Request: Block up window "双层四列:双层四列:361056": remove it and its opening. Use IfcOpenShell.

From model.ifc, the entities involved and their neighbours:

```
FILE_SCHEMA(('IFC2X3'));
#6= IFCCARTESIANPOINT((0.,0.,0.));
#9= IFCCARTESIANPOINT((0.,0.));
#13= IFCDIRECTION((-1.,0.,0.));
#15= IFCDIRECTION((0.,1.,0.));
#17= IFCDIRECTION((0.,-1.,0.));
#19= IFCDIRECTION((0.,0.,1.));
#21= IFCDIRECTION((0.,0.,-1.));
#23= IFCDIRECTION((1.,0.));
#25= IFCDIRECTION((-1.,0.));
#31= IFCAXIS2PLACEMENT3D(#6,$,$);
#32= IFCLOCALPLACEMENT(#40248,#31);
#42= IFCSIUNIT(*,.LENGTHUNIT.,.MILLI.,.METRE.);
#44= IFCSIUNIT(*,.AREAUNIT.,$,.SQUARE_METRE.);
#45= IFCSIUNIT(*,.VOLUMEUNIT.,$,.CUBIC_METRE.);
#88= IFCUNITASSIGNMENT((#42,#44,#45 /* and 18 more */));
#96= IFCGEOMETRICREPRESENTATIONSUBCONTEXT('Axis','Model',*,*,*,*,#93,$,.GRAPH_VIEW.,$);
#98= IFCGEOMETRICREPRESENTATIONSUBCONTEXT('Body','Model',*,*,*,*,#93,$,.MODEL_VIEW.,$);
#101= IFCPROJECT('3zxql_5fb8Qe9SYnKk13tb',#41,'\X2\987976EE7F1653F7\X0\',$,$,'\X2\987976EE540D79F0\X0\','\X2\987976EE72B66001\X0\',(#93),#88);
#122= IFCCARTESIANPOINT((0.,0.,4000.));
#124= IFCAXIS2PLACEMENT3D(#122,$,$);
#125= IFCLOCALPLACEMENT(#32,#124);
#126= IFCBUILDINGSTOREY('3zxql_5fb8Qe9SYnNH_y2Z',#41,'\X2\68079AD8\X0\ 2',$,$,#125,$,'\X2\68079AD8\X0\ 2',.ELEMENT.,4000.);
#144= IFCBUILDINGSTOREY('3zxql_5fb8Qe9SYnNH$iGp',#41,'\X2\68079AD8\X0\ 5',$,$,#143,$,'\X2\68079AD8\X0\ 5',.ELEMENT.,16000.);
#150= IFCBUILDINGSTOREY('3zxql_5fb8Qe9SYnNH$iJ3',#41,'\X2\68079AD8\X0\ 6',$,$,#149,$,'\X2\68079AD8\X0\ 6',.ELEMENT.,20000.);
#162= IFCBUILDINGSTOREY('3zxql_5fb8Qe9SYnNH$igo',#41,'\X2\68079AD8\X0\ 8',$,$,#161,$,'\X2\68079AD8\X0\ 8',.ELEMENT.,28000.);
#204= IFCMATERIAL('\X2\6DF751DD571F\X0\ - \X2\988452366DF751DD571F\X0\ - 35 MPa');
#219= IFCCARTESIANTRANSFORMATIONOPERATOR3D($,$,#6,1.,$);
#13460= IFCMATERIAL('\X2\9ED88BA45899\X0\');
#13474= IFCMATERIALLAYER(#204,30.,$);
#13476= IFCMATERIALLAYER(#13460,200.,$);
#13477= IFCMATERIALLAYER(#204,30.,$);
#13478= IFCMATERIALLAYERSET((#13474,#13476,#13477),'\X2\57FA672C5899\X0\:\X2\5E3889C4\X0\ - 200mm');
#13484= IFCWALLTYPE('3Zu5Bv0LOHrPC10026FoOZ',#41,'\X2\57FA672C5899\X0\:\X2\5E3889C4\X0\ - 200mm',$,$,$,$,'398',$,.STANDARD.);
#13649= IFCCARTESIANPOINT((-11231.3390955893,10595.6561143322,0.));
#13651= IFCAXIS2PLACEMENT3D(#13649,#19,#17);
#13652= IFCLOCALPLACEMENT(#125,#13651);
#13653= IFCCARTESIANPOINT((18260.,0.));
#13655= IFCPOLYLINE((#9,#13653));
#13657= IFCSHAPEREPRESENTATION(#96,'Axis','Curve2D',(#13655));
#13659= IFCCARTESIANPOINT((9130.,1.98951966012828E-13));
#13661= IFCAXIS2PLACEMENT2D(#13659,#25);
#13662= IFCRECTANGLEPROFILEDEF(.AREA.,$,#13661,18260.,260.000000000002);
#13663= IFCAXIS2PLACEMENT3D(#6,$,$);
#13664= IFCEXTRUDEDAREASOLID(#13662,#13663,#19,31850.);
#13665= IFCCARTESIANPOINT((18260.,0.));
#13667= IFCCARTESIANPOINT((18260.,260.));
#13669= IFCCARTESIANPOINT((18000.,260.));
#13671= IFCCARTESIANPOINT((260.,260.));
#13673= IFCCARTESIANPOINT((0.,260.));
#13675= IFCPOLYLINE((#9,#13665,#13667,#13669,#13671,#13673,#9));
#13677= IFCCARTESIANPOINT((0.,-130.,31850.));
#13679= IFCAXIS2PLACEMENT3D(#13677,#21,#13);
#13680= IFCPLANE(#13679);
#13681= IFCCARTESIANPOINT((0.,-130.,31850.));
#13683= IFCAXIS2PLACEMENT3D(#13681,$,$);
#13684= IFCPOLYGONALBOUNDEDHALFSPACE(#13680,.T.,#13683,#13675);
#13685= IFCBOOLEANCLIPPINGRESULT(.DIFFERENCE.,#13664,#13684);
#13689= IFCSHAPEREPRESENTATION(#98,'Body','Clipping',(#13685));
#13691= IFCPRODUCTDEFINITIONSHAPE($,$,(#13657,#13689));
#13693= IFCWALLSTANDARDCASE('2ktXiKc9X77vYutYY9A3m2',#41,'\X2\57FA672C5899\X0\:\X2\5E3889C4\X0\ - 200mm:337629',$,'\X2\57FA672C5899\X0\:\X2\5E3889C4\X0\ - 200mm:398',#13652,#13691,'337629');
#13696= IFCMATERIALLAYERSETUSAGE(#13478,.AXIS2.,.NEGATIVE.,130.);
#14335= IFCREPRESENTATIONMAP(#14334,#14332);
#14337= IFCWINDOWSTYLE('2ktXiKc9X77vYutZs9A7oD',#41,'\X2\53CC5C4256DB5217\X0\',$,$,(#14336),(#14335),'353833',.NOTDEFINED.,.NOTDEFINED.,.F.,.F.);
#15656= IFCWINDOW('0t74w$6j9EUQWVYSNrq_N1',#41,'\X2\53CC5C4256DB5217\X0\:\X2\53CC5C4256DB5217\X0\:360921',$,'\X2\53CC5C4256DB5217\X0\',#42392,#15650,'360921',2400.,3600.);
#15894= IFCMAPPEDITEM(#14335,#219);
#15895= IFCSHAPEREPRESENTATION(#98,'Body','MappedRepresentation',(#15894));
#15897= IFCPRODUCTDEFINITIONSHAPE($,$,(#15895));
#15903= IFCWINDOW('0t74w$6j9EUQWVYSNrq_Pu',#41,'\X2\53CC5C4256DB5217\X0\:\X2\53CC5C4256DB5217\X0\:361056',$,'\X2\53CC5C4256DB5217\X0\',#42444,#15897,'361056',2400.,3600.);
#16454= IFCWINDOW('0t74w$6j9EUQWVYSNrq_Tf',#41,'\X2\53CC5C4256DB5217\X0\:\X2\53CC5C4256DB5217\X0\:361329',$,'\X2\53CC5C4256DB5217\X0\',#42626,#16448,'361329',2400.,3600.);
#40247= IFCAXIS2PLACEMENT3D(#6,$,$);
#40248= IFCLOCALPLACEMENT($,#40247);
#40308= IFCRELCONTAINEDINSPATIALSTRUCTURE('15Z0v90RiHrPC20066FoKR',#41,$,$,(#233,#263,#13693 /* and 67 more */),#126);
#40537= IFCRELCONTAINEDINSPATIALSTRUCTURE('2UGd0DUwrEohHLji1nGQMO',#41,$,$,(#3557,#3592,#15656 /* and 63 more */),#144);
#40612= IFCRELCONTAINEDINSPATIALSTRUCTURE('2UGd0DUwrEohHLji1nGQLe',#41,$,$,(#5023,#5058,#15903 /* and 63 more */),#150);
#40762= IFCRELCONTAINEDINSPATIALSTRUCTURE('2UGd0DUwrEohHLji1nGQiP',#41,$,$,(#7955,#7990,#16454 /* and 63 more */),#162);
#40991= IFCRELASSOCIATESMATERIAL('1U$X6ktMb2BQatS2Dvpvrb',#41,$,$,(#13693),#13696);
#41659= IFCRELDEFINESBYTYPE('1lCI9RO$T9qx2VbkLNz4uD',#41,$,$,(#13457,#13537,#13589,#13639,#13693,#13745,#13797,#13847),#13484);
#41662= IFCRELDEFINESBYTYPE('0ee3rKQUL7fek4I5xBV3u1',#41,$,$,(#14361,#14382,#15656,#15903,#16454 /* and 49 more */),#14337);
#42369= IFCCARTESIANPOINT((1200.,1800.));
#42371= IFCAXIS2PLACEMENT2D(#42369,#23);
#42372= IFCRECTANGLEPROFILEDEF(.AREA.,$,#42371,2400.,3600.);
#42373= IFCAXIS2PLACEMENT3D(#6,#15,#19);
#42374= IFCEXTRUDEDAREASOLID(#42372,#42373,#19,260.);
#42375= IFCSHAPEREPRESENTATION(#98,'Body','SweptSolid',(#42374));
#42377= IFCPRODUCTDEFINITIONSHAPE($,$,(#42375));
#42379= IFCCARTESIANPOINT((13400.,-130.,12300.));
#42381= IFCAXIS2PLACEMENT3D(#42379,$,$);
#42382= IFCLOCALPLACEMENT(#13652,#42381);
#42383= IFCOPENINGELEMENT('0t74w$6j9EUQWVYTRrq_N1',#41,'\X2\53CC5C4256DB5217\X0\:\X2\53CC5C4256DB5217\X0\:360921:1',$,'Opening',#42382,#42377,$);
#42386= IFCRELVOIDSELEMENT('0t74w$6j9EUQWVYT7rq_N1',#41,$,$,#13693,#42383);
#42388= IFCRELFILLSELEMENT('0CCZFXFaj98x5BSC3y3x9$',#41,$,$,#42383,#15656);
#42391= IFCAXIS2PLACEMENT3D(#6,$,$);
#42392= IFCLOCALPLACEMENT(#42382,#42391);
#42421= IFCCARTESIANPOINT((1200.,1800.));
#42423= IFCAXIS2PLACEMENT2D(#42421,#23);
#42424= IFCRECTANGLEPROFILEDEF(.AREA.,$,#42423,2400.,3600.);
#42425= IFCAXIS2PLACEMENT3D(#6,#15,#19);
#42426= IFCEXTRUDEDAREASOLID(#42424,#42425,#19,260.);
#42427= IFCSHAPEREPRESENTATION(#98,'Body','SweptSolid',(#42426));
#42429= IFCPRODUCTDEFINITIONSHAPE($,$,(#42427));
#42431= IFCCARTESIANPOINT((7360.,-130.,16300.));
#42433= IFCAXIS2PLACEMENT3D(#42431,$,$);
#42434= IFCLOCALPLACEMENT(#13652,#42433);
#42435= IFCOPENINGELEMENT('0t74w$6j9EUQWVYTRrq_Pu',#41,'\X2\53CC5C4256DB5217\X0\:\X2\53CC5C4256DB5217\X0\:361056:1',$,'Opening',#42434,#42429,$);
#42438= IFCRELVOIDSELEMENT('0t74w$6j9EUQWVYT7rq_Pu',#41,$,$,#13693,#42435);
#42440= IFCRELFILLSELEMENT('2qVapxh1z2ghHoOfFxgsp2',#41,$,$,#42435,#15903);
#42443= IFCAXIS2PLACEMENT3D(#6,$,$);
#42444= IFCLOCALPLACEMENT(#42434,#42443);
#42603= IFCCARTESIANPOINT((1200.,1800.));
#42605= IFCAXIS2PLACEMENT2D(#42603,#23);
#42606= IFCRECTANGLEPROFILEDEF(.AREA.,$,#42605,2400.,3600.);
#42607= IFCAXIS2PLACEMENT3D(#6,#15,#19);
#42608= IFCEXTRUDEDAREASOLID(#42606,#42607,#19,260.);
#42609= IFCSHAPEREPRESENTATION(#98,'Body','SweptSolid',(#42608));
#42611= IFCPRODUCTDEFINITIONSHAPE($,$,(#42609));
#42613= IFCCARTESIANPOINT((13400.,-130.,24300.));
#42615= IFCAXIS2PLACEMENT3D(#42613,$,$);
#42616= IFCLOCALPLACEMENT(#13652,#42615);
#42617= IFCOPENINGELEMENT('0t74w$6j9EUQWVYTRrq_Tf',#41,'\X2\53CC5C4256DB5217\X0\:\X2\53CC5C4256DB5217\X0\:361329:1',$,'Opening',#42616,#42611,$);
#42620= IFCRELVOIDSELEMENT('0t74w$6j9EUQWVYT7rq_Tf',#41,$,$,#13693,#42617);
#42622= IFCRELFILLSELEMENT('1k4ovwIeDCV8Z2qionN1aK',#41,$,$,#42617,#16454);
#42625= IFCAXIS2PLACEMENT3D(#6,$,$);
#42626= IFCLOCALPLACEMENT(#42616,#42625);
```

```python
import ifcopenshell
import ifcopenshell.api.feature
import ifcopenshell.api.root
import ifcopenshell.geom
import ifcopenshell.util.shape

model = ifcopenshell.open("model.ifc")
settings = ifcopenshell.geom.settings()


def volume(element):
    """Net volume in cubic metres, openings subtracted."""
    shape = ifcopenshell.geom.create_shape(settings, element)
    return ifcopenshell.util.shape.get_volume(shape.geometry)


window = model.by_guid("0t74w$6j9EUQWVYSNrq_Pu")
opening = window.FillsVoids[0].RelatingOpeningElement
wall = opening.VoidsElements[0].RelatingBuildingElement
before = volume(wall)

ifcopenshell.api.root.remove_product(model, product=window)
ifcopenshell.api.feature.remove_feature(model, feature=opening)

after = volume(wall)

print(f"wall volume {before:.3f} -> {after:.3f} m3")

model.write("model_edited.ifc")
```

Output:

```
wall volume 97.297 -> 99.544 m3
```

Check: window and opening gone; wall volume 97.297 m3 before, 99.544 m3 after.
